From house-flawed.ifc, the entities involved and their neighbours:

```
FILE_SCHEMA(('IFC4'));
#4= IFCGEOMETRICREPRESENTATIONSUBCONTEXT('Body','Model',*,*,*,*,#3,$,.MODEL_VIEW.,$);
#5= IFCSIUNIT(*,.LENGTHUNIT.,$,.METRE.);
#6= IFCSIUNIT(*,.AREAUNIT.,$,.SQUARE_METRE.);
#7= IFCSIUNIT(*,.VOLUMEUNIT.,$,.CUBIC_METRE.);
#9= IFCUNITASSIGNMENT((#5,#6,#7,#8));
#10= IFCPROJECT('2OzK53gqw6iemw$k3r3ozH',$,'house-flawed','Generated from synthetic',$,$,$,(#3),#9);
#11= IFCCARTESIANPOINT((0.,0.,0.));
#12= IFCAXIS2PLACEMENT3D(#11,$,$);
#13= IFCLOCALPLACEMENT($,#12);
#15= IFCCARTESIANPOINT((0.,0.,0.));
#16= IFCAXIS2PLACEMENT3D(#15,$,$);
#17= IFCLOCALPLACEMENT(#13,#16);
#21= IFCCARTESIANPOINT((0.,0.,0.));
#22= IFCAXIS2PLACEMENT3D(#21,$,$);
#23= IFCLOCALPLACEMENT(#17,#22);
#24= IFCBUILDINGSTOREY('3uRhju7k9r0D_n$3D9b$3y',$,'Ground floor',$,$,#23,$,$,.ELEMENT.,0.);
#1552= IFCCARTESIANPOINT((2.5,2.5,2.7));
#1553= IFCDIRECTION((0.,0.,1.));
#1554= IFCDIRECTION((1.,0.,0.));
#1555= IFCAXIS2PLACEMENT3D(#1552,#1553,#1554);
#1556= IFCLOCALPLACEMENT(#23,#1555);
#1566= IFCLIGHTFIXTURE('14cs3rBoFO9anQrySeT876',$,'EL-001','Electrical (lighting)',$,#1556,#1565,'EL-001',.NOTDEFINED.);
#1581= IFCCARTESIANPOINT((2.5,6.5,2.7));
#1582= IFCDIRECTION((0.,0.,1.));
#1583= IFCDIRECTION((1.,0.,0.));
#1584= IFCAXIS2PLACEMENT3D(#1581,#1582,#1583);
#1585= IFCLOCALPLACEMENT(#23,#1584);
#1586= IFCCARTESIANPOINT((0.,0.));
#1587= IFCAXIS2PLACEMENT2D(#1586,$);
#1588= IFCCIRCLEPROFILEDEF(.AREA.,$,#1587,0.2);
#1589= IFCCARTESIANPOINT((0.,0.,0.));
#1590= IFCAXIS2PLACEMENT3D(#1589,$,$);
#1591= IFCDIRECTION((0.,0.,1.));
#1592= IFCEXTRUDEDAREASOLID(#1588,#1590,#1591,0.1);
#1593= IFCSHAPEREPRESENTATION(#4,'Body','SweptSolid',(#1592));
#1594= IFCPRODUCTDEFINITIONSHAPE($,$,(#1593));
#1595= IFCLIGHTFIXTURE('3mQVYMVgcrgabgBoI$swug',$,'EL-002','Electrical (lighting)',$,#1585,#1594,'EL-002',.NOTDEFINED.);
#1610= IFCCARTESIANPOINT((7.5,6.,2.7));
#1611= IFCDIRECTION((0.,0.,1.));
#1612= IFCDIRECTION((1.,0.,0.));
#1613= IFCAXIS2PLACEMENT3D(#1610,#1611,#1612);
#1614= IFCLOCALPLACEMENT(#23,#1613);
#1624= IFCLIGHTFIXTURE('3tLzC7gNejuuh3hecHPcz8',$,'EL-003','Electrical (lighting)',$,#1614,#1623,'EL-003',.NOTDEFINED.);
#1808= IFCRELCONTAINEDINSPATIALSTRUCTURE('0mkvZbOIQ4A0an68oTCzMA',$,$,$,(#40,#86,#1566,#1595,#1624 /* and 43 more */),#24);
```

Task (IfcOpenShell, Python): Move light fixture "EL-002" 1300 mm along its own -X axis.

```python
import ifcopenshell
import ifcopenshell.api.geometry
import ifcopenshell.util.placement

model = ifcopenshell.open("house-flawed.ifc")

item = model.by_guid("3mQVYMVgcrgabgBoI$swug")
matrix = ifcopenshell.util.placement.get_local_placement(item.ObjectPlacement)
matrix[:3, 3] -= matrix[:3, 0] * 1.3
ifcopenshell.api.geometry.edit_object_placement(model, product=item, matrix=matrix, is_si=False)

print(ifcopenshell.util.placement.get_local_placement(item.ObjectPlacement).round(3) + 0.0)

model.write("house-flawed-out.ifc")
```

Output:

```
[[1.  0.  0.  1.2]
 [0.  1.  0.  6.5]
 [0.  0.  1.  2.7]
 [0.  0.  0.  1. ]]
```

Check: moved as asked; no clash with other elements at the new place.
